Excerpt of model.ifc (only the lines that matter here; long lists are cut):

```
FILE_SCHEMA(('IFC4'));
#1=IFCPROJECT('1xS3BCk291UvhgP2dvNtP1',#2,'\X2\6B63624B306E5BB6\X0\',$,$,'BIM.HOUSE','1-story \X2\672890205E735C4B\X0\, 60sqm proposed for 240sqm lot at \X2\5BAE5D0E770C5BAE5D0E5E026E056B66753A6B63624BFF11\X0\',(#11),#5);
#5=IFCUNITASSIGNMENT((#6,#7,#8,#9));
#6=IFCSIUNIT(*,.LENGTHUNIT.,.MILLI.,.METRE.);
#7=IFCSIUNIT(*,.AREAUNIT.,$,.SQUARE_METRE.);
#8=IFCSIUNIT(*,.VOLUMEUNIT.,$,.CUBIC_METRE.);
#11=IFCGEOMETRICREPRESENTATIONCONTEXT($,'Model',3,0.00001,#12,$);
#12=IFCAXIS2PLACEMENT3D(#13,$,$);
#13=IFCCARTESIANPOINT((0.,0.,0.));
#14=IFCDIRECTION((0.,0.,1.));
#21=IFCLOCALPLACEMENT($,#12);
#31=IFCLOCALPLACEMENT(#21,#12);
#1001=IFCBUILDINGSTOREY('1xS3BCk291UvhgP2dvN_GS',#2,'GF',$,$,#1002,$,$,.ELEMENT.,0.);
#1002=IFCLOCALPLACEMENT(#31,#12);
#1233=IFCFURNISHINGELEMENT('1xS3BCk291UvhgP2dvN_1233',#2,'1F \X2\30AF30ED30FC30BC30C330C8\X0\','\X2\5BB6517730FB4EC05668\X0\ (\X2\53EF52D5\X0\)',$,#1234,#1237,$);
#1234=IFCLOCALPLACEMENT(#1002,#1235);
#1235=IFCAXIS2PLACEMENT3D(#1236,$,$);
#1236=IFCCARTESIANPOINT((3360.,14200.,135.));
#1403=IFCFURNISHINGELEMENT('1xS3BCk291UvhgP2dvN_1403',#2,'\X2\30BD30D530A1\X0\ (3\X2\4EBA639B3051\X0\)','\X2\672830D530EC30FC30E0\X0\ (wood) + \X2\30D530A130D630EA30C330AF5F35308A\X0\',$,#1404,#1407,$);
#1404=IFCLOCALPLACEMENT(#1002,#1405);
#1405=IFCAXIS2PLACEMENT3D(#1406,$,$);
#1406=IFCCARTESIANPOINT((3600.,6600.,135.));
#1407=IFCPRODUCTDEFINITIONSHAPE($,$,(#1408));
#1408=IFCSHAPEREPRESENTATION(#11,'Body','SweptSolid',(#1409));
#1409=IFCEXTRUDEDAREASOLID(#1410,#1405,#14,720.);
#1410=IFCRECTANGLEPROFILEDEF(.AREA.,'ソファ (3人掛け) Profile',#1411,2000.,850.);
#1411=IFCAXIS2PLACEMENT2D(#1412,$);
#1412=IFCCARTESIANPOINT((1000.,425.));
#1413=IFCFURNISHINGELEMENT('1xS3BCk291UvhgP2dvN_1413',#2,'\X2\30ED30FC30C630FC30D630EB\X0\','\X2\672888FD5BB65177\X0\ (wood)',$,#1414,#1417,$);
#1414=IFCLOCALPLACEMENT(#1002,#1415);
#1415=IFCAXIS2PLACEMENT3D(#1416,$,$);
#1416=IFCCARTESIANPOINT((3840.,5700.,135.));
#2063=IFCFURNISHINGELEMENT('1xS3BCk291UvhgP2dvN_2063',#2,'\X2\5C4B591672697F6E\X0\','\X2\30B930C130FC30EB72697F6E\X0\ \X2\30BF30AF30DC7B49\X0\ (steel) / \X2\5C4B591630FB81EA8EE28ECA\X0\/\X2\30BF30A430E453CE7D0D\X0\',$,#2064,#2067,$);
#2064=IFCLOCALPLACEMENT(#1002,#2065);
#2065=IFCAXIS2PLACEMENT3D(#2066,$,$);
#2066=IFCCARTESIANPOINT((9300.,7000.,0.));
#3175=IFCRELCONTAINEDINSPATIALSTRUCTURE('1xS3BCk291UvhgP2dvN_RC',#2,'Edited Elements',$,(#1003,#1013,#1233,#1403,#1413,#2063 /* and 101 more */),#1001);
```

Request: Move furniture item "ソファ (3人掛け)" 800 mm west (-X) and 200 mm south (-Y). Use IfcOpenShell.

```python
import ifcopenshell
import ifcopenshell.api.geometry
import ifcopenshell.util.placement
import ifcopenshell.util.unit

model = ifcopenshell.open("model.ifc")
unit_scale = ifcopenshell.util.unit.calculate_unit_scale(model)

item = model.by_guid("1xS3BCk291UvhgP2dvN_1403")
matrix = ifcopenshell.util.placement.get_local_placement(item.ObjectPlacement)
matrix[0, 3] -= 0.8 / unit_scale
matrix[1, 3] -= 0.2 / unit_scale
ifcopenshell.api.geometry.edit_object_placement(model, product=item, matrix=matrix, is_si=False)

print(ifcopenshell.util.placement.get_local_placement(item.ObjectPlacement).round(3) + 0.0)

model.write("model_rev.ifc")
```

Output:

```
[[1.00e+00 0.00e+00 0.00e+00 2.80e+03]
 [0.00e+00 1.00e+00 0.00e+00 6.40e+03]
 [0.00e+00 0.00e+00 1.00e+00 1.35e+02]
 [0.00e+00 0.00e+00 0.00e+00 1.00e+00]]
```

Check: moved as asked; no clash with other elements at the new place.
